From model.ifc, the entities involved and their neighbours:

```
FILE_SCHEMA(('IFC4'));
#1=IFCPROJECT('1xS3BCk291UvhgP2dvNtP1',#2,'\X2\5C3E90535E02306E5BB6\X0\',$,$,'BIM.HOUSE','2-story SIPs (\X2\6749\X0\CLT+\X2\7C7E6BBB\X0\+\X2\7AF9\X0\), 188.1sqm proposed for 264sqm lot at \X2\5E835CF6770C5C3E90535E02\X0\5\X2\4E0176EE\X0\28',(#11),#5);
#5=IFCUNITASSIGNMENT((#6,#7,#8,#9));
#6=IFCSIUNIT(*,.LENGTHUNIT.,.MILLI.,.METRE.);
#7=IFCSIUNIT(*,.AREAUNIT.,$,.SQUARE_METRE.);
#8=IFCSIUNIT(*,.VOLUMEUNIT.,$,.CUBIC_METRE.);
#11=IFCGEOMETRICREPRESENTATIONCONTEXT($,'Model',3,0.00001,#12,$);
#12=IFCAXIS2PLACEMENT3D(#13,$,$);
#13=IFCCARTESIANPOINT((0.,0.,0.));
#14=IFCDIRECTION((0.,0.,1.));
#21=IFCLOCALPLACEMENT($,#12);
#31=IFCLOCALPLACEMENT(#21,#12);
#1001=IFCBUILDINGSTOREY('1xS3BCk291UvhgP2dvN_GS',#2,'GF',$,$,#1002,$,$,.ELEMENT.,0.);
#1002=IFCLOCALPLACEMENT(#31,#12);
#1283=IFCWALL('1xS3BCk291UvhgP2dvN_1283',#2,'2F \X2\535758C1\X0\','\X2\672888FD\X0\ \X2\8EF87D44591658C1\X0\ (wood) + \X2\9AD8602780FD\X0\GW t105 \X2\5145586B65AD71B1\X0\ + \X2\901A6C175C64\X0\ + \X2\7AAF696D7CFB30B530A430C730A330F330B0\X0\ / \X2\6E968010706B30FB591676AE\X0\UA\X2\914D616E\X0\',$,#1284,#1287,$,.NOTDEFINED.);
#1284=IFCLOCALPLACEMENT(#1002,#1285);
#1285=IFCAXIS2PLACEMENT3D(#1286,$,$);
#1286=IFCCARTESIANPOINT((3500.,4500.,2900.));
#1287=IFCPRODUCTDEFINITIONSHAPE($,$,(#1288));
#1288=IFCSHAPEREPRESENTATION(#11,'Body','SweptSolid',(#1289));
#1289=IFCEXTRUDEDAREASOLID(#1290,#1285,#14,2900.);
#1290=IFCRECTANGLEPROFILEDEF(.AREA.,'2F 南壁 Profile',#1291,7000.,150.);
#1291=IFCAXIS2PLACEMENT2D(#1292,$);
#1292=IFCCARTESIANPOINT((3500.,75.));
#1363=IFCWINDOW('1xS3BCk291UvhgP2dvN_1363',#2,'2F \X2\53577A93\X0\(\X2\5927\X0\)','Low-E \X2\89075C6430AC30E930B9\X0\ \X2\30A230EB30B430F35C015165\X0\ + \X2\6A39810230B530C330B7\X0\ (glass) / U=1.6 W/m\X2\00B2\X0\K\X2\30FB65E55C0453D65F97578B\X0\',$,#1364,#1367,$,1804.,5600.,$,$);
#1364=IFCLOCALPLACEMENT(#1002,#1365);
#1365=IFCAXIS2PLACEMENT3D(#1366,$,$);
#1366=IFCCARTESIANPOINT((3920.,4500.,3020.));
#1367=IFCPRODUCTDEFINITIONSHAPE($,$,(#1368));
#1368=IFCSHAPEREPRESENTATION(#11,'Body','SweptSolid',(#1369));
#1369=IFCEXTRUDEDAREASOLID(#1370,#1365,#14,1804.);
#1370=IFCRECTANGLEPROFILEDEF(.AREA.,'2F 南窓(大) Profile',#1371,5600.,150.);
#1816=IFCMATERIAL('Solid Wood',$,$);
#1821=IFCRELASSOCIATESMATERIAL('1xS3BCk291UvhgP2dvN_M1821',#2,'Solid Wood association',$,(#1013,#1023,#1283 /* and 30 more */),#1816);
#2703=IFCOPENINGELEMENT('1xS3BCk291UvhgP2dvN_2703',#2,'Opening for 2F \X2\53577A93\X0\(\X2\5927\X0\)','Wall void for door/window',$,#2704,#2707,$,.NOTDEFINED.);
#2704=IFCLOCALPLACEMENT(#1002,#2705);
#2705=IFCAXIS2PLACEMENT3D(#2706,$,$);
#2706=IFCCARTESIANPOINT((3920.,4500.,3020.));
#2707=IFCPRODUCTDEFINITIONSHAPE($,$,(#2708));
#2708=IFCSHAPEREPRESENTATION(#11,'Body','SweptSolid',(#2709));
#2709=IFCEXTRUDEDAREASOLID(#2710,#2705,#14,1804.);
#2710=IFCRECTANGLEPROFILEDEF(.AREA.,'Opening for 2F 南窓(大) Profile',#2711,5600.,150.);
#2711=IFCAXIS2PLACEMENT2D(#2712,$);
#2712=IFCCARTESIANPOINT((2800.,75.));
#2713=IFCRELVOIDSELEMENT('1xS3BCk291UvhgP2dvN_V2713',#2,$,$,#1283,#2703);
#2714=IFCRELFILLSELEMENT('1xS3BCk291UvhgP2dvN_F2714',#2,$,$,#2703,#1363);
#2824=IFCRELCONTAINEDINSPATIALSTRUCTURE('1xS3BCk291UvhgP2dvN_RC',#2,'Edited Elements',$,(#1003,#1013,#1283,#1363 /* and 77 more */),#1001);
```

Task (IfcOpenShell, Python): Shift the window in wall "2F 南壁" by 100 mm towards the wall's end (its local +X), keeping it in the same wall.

```python
import ifcopenshell
import ifcopenshell.api.geometry
import ifcopenshell.util.placement
import ifcopenshell.util.unit

model = ifcopenshell.open("model.ifc")
unit_scale = ifcopenshell.util.unit.calculate_unit_scale(model)

window = model.by_guid("1xS3BCk291UvhgP2dvN_1363")
opening = window.FillsVoids[0].RelatingOpeningElement
wall = opening.VoidsElements[0].RelatingBuildingElement

wall_matrix = ifcopenshell.util.placement.get_local_placement(wall.ObjectPlacement)
shift = wall_matrix[:3, 0] * 0.1 / unit_scale
before = ifcopenshell.util.placement.get_local_placement(window.ObjectPlacement)[:3, 3].copy()

# The window is not placed relative to its opening, so move both.
for product in (opening, window):
    matrix = ifcopenshell.util.placement.get_local_placement(product.ObjectPlacement)
    matrix[:3, 3] += shift
    ifcopenshell.api.geometry.edit_object_placement(model, product=product, matrix=matrix, is_si=False)

after = ifcopenshell.util.placement.get_local_placement(window.ObjectPlacement)[:3, 3]
print("window moved by", (after - before).round(3) + 0.0)

model.write("model_updated.ifc")
```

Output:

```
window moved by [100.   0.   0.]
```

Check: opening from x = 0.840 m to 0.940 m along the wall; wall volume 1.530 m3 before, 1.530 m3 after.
